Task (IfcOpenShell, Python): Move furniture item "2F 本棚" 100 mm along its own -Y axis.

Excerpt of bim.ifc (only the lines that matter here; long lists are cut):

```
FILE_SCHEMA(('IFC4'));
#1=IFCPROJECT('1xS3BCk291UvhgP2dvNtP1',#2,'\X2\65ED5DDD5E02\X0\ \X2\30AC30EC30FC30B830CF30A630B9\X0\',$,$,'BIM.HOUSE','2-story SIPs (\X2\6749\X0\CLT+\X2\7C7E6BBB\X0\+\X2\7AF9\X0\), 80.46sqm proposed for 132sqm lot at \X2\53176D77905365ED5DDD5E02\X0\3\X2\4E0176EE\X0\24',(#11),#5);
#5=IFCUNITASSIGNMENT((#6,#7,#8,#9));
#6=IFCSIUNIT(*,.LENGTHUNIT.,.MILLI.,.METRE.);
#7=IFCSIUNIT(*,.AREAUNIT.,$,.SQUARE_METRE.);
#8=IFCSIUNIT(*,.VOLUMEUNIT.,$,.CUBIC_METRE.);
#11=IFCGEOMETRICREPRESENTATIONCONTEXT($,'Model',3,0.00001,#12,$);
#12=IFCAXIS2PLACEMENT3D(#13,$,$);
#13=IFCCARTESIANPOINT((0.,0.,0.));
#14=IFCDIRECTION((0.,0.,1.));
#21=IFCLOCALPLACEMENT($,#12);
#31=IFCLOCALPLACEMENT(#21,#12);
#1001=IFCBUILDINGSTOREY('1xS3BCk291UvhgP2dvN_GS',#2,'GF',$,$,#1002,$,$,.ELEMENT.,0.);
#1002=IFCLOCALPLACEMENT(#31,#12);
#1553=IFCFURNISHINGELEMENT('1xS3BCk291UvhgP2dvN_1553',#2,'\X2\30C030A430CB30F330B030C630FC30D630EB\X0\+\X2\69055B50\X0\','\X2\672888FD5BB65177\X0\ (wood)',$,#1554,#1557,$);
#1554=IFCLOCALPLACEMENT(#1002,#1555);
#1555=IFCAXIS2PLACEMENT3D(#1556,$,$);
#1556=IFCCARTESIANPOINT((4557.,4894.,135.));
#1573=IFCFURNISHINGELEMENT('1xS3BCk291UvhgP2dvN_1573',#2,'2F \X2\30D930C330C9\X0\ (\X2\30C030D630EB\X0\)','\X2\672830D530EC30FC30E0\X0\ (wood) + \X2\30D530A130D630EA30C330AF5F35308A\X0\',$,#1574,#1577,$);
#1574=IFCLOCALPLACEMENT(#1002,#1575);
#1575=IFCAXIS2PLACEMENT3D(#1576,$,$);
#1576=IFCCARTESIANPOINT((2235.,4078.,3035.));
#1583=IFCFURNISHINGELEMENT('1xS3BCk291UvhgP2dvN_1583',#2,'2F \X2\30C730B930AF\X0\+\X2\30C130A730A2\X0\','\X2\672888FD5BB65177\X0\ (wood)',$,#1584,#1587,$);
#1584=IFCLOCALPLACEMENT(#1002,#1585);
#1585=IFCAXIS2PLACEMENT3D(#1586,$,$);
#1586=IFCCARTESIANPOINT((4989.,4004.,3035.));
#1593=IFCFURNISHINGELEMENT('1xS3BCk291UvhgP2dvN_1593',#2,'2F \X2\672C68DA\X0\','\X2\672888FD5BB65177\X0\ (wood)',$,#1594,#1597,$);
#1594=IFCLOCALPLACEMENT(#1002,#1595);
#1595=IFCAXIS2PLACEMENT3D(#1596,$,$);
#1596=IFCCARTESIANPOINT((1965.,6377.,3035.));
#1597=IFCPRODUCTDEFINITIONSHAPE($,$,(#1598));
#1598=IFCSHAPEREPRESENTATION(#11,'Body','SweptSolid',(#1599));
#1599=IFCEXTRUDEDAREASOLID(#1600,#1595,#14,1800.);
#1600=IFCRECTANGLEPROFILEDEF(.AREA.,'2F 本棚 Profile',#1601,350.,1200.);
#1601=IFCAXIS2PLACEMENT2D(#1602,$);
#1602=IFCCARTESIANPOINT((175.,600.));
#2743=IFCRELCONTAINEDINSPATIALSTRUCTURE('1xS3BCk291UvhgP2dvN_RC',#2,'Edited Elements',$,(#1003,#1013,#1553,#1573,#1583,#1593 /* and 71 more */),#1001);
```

```python
import ifcopenshell
import ifcopenshell.api.geometry
import ifcopenshell.util.placement
import ifcopenshell.util.unit

model = ifcopenshell.open("bim.ifc")
unit_scale = ifcopenshell.util.unit.calculate_unit_scale(model)

item = model.by_guid("1xS3BCk291UvhgP2dvN_1593")
matrix = ifcopenshell.util.placement.get_local_placement(item.ObjectPlacement)
matrix[:3, 3] -= matrix[:3, 1] * 0.1 / unit_scale
ifcopenshell.api.geometry.edit_object_placement(model, product=item, matrix=matrix, is_si=False)

print(ifcopenshell.util.placement.get_local_placement(item.ObjectPlacement).round(3) + 0.0)

model.write("bim_v2.ifc")
```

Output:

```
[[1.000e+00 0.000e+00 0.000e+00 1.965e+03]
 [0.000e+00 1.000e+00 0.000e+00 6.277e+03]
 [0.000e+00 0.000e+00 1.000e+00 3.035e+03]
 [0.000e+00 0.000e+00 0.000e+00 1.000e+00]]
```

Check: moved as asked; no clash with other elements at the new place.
